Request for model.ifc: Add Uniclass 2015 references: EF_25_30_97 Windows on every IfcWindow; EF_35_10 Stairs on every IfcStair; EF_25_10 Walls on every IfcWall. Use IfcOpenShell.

First a look at what the model holds.

```python
import ifcopenshell

model = ifcopenshell.open("model.ifc")
print(model.schema)
print("classifications:", [c.Name for c in model.by_type("IfcClassification")])
for ifc_class in ("IfcDoor", "IfcRoof", "IfcStair", "IfcWall", "IfcWindow"):
    print(ifc_class, len(model.by_type(ifc_class)))
```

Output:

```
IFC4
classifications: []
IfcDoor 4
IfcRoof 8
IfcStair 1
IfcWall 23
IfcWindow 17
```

```python
import ifcopenshell
import ifcopenshell.api.classification

model = ifcopenshell.open("model.ifc")

system = ifcopenshell.api.classification.add_classification(model, classification="Uniclass 2015")

codes = {
    "IfcWindow": ("EF_25_30_97", "Windows"),
    "IfcStair": ("EF_35_10", "Stairs"),
    "IfcWall": ("EF_25_10", "Walls"),
}
for ifc_class, (code, name) in codes.items():
    products = model.by_type(ifc_class)
    ifcopenshell.api.classification.add_reference(
        model, products=products, classification=system, identification=code, name=name
    )
    print(code, len(products))

model.write("model_updated.ifc")
```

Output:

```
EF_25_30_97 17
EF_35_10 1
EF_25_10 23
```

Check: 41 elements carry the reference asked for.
